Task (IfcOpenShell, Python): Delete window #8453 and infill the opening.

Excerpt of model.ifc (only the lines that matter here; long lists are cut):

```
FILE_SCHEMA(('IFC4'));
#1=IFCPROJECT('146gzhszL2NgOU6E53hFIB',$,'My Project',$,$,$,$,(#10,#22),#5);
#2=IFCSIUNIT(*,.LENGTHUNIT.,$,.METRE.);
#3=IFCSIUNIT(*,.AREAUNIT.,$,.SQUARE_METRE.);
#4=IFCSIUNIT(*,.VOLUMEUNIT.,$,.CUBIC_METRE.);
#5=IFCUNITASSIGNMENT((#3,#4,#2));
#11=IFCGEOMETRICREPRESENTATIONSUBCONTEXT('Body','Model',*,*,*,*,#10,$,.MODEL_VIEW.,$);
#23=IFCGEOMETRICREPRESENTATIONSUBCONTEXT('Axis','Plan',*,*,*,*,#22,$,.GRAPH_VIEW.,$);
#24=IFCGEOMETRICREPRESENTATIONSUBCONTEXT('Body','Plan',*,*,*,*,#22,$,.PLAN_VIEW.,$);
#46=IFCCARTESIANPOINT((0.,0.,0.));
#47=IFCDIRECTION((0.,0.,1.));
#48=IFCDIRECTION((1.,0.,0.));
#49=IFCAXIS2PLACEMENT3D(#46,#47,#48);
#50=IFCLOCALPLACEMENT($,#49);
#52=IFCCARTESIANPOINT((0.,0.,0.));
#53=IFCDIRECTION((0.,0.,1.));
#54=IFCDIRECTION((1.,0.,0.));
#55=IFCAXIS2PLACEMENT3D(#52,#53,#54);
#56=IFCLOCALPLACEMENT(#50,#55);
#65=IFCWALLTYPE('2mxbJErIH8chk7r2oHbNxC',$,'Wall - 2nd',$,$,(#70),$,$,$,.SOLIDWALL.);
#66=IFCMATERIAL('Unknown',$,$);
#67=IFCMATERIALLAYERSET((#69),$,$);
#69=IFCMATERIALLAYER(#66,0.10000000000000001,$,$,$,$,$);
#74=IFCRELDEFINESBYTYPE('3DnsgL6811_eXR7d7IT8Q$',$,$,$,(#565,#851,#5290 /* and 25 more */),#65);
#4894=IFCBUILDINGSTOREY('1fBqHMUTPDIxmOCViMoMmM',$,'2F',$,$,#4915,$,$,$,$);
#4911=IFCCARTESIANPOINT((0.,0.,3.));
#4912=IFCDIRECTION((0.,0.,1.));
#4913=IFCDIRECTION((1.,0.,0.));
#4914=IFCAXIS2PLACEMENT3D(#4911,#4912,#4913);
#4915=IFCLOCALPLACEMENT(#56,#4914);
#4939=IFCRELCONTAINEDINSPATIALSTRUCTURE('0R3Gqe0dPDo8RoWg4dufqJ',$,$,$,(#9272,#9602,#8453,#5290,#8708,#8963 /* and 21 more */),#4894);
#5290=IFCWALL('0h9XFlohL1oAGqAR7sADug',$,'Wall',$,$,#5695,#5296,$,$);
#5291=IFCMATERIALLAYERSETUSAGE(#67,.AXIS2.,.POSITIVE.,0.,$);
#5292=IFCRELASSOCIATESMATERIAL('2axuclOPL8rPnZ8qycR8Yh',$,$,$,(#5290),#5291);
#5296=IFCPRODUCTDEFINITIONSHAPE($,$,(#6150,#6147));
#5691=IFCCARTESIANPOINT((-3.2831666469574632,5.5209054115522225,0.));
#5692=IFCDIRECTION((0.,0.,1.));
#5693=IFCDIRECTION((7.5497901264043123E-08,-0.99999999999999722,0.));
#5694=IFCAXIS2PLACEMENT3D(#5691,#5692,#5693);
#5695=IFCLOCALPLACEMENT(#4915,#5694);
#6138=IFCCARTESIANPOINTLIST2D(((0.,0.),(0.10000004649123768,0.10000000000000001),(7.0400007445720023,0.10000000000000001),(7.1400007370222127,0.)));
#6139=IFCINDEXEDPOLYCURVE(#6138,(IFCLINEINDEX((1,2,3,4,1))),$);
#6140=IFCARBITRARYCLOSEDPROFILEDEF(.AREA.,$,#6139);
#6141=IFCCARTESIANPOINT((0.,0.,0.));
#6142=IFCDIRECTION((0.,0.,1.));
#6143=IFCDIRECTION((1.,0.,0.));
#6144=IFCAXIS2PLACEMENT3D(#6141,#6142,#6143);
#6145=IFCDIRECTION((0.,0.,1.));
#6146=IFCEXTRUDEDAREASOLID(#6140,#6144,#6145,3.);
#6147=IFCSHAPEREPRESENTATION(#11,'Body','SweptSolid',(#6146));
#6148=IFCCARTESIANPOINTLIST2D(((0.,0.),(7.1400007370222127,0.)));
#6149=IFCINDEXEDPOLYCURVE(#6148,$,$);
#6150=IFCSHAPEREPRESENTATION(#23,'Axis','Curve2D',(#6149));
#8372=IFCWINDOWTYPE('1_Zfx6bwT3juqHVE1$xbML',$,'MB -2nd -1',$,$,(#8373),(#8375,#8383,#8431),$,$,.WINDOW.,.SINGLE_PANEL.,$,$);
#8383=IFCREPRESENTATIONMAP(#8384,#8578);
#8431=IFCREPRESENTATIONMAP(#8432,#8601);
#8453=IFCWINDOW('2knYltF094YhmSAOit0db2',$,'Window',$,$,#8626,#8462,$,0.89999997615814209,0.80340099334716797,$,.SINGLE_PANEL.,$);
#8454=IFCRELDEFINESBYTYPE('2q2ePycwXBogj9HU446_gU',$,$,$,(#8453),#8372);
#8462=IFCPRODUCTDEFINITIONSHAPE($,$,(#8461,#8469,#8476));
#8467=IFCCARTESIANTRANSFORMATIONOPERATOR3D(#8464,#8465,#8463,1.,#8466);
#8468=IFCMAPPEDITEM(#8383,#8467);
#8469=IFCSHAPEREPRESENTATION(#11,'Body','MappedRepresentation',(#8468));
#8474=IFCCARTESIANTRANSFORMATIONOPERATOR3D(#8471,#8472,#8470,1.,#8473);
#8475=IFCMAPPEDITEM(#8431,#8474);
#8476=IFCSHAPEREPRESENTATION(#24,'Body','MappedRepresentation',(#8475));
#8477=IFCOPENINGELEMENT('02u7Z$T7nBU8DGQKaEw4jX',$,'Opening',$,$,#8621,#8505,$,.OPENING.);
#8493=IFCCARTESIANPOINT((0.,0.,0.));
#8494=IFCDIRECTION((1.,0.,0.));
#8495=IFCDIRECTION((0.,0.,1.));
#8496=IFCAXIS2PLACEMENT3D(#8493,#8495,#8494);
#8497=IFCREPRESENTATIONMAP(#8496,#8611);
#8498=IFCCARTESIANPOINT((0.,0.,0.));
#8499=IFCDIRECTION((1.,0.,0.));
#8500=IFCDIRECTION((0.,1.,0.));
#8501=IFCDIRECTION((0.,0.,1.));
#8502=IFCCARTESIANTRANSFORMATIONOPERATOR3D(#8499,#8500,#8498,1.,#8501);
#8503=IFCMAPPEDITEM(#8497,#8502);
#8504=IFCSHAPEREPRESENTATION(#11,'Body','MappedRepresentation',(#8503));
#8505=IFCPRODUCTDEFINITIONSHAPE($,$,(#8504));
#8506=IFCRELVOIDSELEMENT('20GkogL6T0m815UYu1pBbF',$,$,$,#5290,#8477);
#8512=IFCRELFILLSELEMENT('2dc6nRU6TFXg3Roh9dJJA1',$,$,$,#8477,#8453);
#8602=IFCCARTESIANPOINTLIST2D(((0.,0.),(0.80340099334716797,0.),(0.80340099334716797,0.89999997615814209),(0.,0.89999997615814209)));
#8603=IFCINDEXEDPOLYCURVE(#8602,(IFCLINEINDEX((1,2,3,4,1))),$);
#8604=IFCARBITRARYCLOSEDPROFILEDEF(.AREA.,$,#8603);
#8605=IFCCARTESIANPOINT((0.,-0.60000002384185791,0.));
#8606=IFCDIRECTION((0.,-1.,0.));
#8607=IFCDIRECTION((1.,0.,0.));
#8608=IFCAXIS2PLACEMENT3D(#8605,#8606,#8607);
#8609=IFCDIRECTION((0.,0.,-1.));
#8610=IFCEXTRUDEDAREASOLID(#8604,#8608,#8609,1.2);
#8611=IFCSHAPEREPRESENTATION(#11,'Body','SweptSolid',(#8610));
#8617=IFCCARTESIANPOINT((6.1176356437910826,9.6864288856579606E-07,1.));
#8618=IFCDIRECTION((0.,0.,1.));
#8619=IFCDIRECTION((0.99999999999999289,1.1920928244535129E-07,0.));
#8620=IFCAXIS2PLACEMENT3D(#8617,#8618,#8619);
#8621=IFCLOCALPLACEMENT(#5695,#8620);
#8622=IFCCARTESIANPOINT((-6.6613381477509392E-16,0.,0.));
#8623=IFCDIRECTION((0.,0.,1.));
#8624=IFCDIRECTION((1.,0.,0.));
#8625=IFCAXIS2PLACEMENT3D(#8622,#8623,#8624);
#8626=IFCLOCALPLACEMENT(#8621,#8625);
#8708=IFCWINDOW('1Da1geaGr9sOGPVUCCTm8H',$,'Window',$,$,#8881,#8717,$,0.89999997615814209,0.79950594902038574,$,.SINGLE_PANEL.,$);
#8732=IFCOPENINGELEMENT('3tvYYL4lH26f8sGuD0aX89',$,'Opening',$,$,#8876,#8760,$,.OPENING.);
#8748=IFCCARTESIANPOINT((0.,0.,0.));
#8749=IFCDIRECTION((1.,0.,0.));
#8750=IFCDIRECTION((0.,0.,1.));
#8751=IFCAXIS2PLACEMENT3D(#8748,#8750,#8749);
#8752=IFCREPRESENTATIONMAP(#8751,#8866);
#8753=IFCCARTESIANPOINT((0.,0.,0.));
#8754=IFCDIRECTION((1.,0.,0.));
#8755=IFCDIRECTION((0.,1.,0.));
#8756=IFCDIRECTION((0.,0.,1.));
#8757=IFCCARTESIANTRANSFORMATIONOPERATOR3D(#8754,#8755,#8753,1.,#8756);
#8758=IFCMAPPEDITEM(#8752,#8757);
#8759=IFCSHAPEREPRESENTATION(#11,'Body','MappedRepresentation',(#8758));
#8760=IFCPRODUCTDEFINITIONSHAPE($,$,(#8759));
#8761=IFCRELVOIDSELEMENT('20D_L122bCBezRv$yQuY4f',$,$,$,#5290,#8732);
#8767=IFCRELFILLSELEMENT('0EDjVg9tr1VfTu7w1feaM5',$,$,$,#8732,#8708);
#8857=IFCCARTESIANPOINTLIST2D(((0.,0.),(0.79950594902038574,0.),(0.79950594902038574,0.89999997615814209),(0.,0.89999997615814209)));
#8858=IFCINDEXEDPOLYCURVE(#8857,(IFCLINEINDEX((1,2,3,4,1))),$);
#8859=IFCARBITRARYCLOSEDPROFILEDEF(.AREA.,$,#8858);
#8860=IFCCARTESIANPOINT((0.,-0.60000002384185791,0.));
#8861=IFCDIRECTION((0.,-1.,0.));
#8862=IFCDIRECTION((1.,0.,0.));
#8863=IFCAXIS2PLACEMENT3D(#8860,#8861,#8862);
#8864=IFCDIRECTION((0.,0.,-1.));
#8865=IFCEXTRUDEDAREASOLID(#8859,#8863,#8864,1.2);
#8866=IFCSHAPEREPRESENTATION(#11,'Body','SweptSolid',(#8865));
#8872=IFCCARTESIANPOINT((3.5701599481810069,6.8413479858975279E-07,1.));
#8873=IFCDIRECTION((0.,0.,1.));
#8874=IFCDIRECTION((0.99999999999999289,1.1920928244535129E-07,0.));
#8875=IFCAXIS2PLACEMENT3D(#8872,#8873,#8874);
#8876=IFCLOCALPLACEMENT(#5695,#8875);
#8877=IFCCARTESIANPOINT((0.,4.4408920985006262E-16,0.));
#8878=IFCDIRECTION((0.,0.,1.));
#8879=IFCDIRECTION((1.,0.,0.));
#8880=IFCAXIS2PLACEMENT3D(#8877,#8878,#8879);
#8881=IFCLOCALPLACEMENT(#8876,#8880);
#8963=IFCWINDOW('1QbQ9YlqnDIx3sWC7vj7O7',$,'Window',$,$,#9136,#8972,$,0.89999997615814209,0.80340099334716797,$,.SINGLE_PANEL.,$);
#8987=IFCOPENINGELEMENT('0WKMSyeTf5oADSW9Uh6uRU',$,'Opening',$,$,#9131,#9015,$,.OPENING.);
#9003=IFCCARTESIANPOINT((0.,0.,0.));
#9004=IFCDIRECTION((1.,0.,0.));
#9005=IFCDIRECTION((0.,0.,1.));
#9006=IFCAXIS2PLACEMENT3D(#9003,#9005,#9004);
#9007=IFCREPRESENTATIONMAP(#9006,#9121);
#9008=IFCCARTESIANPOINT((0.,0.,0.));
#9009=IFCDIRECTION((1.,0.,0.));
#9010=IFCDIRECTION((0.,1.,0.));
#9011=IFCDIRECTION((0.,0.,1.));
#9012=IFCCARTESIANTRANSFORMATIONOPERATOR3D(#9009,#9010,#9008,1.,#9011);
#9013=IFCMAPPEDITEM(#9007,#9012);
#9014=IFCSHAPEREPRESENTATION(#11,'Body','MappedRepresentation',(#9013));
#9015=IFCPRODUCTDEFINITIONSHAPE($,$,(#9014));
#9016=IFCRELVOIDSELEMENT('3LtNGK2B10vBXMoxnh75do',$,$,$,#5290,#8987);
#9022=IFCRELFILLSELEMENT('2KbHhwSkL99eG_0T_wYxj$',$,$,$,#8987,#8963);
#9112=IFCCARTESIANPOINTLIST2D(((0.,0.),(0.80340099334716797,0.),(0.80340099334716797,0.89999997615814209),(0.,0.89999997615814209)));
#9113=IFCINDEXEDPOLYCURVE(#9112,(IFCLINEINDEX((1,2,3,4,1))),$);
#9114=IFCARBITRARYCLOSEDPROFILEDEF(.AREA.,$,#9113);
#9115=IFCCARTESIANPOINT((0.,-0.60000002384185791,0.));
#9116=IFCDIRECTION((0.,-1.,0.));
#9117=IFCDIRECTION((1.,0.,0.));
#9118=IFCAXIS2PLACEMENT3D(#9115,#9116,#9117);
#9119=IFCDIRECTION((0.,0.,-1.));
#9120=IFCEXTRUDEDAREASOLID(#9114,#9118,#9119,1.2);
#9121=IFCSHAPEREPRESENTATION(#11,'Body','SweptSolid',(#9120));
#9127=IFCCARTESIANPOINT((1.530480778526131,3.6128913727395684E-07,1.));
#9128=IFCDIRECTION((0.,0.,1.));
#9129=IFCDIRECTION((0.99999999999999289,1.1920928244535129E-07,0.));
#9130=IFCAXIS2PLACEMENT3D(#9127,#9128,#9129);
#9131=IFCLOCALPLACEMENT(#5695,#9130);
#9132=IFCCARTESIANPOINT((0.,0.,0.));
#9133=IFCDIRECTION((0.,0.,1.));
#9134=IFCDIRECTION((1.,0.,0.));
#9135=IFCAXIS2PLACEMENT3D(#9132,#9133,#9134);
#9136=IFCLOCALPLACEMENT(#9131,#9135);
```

```python
import ifcopenshell
import ifcopenshell.api.feature
import ifcopenshell.api.root
import ifcopenshell.geom
import ifcopenshell.util.shape

model = ifcopenshell.open("model.ifc")
settings = ifcopenshell.geom.settings()


def volume(element):
    """Net volume in cubic metres, openings subtracted."""
    shape = ifcopenshell.geom.create_shape(settings, element)
    return ifcopenshell.util.shape.get_volume(shape.geometry)


window = model.by_guid("2knYltF094YhmSAOit0db2")
opening = window.FillsVoids[0].RelatingOpeningElement
wall = opening.VoidsElements[0].RelatingBuildingElement
before = volume(wall)

ifcopenshell.api.root.remove_product(model, product=window)
ifcopenshell.api.feature.remove_feature(model, feature=opening)

after = volume(wall)

print(f"wall volume {before:.3f} -> {after:.3f} m3")

model.write("model-out.ifc")
```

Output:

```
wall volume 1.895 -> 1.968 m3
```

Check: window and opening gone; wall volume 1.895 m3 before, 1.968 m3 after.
